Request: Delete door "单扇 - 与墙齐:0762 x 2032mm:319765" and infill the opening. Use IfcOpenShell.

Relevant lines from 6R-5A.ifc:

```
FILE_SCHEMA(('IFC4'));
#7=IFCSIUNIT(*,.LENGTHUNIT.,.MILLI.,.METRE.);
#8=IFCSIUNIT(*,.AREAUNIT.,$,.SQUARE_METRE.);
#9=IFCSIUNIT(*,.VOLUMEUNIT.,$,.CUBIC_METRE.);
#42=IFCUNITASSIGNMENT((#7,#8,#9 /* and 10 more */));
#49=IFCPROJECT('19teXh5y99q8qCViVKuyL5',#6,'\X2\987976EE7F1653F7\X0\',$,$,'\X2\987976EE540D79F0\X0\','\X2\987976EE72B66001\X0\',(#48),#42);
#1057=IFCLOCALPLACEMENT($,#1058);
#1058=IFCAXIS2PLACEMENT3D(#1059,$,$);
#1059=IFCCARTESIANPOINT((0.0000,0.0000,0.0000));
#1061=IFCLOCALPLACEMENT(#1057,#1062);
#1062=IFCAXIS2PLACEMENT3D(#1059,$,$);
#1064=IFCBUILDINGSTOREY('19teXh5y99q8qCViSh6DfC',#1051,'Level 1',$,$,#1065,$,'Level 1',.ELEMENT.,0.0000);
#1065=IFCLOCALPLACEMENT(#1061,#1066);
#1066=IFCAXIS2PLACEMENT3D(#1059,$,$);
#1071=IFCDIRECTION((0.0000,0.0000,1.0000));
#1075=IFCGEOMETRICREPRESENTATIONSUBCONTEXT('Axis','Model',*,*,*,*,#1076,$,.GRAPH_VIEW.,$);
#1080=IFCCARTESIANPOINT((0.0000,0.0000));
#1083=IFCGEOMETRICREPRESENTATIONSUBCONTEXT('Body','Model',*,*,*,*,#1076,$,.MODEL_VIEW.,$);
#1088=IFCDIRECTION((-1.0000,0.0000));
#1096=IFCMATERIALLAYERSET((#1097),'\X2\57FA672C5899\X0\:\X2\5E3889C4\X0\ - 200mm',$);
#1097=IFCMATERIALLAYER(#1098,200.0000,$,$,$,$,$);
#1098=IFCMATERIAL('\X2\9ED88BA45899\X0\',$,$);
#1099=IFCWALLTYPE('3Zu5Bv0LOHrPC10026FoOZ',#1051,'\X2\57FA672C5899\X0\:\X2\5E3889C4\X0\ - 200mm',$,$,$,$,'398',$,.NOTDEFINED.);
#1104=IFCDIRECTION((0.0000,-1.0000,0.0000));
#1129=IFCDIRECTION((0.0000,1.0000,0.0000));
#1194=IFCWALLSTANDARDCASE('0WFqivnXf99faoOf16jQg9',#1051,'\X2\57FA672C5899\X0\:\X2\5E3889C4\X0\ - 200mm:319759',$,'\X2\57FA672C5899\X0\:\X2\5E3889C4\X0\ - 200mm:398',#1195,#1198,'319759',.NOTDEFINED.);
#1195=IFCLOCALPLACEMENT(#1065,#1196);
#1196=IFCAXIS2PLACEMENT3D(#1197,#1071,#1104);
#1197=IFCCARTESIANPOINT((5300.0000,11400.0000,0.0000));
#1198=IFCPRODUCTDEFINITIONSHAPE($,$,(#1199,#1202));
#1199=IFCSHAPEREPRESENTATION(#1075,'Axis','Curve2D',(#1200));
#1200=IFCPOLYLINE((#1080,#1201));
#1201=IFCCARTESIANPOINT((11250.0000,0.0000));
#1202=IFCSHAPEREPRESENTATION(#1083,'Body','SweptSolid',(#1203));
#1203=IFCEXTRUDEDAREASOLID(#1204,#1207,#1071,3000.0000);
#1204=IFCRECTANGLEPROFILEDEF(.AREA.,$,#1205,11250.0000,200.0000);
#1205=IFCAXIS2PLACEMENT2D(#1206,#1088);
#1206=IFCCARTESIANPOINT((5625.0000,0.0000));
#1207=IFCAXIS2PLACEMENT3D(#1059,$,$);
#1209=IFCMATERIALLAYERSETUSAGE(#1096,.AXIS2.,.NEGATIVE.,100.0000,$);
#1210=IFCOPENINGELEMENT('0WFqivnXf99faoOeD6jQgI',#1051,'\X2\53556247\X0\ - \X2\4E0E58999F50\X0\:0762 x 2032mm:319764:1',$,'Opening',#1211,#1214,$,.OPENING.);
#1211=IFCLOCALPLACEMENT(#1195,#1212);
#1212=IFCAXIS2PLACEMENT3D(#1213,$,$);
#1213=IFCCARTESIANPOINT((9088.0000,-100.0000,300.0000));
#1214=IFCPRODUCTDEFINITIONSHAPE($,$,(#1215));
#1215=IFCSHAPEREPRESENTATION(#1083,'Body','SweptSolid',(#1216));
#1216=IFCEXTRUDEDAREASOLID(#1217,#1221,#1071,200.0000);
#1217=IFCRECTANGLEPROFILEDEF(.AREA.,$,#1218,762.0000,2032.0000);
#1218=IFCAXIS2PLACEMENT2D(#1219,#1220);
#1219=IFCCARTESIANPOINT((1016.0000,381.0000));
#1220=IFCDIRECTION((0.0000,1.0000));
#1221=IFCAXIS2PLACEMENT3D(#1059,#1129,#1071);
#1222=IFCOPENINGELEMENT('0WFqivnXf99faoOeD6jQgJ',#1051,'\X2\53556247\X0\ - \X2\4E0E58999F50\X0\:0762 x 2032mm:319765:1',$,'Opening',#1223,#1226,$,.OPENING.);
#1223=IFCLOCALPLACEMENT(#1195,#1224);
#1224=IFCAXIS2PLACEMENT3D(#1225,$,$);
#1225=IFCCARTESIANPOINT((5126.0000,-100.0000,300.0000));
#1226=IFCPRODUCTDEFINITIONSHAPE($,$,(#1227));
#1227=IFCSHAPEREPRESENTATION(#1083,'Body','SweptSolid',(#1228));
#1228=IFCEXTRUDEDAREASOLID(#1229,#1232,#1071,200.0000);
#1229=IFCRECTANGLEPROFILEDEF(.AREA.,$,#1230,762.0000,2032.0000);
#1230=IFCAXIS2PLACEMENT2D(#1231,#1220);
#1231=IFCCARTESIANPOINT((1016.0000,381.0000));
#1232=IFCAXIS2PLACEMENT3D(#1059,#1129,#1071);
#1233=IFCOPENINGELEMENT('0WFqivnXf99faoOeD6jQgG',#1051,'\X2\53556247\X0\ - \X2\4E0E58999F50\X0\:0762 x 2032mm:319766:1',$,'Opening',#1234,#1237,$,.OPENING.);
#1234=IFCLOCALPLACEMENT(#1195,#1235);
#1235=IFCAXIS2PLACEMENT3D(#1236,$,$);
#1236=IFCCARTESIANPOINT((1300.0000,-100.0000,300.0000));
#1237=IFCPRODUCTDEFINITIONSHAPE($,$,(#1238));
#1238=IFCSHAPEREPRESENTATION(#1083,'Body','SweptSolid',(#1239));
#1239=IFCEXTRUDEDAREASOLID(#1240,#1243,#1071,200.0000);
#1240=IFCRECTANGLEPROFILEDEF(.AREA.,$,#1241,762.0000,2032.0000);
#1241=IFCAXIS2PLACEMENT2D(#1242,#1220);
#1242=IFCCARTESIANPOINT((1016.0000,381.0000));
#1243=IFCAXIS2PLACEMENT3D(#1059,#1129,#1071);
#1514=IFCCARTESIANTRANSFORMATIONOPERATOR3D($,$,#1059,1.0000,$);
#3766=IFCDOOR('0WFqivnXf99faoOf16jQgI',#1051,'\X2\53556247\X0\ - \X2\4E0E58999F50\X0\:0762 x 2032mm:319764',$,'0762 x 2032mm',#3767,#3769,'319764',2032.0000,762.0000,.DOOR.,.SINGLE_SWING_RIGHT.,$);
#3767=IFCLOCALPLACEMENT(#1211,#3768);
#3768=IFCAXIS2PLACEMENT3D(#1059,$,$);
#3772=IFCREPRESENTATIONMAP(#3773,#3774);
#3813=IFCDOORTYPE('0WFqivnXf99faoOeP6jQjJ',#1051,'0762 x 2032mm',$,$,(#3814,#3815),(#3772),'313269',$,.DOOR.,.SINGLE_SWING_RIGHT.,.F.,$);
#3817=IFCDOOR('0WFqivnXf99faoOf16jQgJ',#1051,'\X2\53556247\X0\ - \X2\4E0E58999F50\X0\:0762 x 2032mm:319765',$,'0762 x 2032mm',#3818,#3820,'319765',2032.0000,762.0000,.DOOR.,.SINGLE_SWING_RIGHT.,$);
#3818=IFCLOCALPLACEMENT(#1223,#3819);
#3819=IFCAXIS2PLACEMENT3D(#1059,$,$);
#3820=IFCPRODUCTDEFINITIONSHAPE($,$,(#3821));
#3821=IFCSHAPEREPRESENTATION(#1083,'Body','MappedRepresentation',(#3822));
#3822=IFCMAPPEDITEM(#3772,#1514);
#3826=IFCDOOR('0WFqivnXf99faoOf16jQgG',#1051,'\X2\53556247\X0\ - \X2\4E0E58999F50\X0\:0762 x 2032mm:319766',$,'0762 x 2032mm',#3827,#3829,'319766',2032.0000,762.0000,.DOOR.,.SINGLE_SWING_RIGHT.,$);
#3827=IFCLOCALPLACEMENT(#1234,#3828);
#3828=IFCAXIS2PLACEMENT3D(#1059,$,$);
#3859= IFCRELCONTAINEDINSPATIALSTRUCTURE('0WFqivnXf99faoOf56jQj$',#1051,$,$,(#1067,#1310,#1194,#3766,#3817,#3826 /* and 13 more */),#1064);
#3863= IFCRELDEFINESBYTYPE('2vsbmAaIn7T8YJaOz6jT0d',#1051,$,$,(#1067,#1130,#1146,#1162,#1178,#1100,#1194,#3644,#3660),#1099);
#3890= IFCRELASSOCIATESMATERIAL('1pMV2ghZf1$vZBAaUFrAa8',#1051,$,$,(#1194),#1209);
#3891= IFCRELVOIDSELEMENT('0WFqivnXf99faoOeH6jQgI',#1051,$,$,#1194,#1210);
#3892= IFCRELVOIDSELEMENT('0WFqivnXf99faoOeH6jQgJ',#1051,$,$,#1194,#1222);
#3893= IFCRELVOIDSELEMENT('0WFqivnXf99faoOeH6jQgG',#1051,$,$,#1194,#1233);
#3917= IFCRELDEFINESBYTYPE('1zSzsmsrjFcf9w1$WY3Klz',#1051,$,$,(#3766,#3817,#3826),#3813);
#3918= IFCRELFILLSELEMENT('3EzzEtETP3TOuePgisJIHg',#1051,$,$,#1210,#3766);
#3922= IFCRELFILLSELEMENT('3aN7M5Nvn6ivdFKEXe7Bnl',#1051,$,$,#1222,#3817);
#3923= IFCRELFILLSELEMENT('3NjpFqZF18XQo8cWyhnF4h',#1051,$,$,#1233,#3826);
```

```python
import ifcopenshell
import ifcopenshell.api.feature
import ifcopenshell.api.root
import ifcopenshell.geom
import ifcopenshell.util.shape

model = ifcopenshell.open("6R-5A.ifc")
settings = ifcopenshell.geom.settings()


def volume(element):
    """Net volume in cubic metres, openings subtracted."""
    shape = ifcopenshell.geom.create_shape(settings, element)
    return ifcopenshell.util.shape.get_volume(shape.geometry)


door = model.by_id(3817)
opening = door.FillsVoids[0].RelatingOpeningElement
wall = opening.VoidsElements[0].RelatingBuildingElement
before = volume(wall)

ifcopenshell.api.root.remove_product(model, product=door)
ifcopenshell.api.feature.remove_feature(model, feature=opening)

after = volume(wall)

print(f"wall volume {before:.3f} -> {after:.3f} m3")

model.write("6R-5A_updated.ifc")
```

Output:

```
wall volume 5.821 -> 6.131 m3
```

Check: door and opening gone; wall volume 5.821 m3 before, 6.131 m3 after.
